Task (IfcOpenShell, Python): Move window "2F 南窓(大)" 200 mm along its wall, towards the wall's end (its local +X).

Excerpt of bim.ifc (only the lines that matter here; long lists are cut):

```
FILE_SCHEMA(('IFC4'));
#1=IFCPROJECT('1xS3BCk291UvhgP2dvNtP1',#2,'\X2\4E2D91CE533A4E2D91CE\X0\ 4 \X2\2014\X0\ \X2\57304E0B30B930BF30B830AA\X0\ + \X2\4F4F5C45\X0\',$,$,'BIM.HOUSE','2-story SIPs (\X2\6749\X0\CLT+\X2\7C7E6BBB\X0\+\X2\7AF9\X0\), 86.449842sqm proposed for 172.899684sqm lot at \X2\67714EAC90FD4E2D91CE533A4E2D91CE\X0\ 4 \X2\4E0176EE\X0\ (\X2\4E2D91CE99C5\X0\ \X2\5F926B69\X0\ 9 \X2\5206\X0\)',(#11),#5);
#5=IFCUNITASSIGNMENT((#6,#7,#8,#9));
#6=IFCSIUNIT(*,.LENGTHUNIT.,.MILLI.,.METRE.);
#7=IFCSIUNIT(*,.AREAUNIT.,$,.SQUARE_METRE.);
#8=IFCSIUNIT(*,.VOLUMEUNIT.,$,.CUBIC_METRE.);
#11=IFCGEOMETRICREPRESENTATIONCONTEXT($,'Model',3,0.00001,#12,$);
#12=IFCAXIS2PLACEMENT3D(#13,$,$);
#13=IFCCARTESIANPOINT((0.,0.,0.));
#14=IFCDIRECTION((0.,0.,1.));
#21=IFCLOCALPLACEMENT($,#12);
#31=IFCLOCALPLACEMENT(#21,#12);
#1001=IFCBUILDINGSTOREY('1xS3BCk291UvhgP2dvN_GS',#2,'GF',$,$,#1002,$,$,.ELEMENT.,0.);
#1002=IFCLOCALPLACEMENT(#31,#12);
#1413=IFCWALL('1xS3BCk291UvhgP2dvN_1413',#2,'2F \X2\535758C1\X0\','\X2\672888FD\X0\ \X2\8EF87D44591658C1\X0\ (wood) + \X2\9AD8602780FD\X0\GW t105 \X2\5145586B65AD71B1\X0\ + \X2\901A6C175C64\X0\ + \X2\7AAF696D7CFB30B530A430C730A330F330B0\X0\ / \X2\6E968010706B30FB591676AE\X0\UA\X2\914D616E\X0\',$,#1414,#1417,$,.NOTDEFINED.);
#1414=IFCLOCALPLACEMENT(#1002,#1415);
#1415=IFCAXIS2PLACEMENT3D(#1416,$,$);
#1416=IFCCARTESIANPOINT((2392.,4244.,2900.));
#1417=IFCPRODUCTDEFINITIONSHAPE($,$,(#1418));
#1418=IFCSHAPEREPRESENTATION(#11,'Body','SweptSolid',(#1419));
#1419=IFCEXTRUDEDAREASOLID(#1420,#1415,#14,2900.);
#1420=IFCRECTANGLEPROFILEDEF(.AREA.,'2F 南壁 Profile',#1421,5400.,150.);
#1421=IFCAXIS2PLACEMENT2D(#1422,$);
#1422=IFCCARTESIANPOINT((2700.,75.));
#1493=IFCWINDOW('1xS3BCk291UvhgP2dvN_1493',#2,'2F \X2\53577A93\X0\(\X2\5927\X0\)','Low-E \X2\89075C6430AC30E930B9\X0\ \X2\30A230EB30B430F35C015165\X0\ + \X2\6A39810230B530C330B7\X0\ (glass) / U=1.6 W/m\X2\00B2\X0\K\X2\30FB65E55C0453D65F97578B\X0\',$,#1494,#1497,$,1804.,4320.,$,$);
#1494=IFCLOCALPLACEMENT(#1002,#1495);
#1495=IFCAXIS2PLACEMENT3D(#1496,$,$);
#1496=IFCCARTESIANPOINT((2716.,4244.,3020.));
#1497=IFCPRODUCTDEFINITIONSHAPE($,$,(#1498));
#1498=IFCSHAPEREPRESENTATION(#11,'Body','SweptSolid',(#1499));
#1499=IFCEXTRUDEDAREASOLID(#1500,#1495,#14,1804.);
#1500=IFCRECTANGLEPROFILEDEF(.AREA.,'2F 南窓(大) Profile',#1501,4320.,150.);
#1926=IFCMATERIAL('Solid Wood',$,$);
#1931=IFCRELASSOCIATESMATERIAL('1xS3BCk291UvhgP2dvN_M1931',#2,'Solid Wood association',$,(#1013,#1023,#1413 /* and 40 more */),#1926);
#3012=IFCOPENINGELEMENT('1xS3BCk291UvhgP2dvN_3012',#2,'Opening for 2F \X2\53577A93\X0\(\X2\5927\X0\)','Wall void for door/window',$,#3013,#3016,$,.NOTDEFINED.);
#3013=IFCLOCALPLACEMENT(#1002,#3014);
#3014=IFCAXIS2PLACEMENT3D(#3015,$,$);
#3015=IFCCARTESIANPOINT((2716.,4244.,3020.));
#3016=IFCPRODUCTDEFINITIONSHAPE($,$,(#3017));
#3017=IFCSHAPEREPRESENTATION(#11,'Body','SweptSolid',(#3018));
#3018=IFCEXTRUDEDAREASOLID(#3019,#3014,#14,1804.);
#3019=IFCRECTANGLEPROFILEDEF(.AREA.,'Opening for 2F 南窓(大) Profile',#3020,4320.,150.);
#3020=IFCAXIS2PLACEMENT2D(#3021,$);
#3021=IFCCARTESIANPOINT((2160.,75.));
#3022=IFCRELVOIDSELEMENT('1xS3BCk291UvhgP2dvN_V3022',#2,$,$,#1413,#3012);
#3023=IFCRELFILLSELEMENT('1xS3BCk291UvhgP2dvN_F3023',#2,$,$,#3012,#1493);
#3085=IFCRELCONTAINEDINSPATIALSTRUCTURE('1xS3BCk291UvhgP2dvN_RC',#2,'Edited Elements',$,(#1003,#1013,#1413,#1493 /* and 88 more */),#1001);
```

```python
import ifcopenshell
import ifcopenshell.api.geometry
import ifcopenshell.util.placement
import ifcopenshell.util.unit

model = ifcopenshell.open("bim.ifc")
unit_scale = ifcopenshell.util.unit.calculate_unit_scale(model)

window = model.by_guid("1xS3BCk291UvhgP2dvN_1493")
opening = window.FillsVoids[0].RelatingOpeningElement
wall = opening.VoidsElements[0].RelatingBuildingElement

wall_matrix = ifcopenshell.util.placement.get_local_placement(wall.ObjectPlacement)
shift = wall_matrix[:3, 0] * 0.2 / unit_scale
before = ifcopenshell.util.placement.get_local_placement(window.ObjectPlacement)[:3, 3].copy()

# The window is not placed relative to its opening, so move both.
for product in (opening, window):
    matrix = ifcopenshell.util.placement.get_local_placement(product.ObjectPlacement)
    matrix[:3, 3] += shift
    ifcopenshell.api.geometry.edit_object_placement(model, product=product, matrix=matrix, is_si=False)

after = ifcopenshell.util.placement.get_local_placement(window.ObjectPlacement)[:3, 3]
print("window moved by", (after - before).round(3) + 0.0)

model.write("bim_rev.ifc")
```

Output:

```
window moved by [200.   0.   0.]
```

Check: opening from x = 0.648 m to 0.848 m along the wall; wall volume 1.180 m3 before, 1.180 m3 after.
